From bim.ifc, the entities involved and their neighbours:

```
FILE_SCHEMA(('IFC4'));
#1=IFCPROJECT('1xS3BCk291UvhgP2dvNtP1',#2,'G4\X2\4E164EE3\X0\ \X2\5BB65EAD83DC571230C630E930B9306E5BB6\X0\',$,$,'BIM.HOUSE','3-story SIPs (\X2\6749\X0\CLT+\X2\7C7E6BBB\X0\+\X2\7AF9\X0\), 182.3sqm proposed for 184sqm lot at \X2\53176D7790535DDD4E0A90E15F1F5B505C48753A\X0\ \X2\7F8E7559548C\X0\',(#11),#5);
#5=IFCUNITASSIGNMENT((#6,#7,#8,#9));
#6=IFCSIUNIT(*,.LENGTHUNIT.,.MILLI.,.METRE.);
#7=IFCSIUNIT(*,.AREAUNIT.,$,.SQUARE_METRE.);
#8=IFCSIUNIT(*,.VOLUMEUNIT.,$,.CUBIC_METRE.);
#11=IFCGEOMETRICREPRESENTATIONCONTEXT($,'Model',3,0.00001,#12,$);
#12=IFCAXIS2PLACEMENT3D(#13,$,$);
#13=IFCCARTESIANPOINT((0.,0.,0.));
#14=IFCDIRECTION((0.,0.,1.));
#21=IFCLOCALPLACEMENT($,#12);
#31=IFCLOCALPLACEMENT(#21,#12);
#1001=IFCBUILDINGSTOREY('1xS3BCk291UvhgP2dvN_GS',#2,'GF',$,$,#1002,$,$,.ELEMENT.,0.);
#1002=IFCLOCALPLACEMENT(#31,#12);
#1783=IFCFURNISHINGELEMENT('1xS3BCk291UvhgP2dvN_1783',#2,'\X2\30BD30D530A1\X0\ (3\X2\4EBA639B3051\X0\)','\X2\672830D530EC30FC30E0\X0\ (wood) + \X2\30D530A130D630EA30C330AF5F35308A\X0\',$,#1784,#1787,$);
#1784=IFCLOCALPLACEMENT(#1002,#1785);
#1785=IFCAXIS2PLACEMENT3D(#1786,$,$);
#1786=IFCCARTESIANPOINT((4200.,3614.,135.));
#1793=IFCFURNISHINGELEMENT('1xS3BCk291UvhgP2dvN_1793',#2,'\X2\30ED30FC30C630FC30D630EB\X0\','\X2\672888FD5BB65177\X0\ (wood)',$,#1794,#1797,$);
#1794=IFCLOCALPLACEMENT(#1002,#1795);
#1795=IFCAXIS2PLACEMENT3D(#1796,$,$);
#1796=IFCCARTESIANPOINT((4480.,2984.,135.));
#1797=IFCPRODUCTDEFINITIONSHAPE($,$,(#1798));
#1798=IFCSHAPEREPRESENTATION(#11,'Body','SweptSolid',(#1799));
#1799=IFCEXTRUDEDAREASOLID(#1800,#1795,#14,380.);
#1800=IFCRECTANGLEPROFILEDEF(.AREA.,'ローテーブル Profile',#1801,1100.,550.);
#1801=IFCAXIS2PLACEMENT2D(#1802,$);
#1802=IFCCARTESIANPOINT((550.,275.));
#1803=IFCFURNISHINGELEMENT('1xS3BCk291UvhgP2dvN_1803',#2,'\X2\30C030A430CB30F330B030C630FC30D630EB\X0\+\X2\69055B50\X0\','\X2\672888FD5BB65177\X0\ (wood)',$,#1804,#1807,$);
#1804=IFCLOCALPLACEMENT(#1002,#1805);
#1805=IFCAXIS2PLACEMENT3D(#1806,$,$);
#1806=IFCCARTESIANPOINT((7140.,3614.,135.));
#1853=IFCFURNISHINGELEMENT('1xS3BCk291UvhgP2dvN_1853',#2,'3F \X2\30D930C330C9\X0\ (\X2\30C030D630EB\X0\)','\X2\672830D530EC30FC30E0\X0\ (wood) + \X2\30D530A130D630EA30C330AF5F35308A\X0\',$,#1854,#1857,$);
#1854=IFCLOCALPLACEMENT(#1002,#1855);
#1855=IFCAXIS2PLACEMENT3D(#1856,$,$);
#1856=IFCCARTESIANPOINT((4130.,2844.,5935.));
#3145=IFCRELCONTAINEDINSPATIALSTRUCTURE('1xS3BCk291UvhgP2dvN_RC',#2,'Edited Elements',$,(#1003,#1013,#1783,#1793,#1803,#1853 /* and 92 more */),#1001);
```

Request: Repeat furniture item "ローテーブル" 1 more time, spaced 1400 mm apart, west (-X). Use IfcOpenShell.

```python
import numpy as np
import ifcopenshell
import ifcopenshell.api.geometry
import ifcopenshell.api.root
import ifcopenshell.util.element
import ifcopenshell.util.placement

model = ifcopenshell.open("bim.ifc")


def reuse_history(source, copy):
    """copy_class also copies each property set's owner history, people and application; keep the originals."""
    for rel in copy.IsDefinedBy:
        if rel.is_a("IfcRelDefinesByProperties") and (history := rel.RelatingPropertyDefinition.OwnerHistory):
            rel.RelatingPropertyDefinition.OwnerHistory = source.OwnerHistory
            ifcopenshell.util.element.remove_deep2(model, history)


source = model.by_guid("1xS3BCk291UvhgP2dvN_1793")
base = ifcopenshell.util.placement.get_local_placement(source.ObjectPlacement)
step = np.array([-1.0, 0.0, 0.0]) * 1400.0

for i in range(1, 2):
    copy = ifcopenshell.api.root.copy_class(model, product=source)
    copy.Representation = ifcopenshell.util.element.copy_deep(
        model, source.Representation, exclude=["IfcGeometricRepresentationContext", "IfcRepresentationMap"]
    )
    reuse_history(source, copy)
    matrix = base.copy()
    matrix[:3, 3] += i * step
    print("added at", matrix[:3, 3].round(3) + 0.0)
    ifcopenshell.api.geometry.edit_object_placement(model, product=copy, matrix=matrix, is_si=False)

model.write("bim-out.ifc")
```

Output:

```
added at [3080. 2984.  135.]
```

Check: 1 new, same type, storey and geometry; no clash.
